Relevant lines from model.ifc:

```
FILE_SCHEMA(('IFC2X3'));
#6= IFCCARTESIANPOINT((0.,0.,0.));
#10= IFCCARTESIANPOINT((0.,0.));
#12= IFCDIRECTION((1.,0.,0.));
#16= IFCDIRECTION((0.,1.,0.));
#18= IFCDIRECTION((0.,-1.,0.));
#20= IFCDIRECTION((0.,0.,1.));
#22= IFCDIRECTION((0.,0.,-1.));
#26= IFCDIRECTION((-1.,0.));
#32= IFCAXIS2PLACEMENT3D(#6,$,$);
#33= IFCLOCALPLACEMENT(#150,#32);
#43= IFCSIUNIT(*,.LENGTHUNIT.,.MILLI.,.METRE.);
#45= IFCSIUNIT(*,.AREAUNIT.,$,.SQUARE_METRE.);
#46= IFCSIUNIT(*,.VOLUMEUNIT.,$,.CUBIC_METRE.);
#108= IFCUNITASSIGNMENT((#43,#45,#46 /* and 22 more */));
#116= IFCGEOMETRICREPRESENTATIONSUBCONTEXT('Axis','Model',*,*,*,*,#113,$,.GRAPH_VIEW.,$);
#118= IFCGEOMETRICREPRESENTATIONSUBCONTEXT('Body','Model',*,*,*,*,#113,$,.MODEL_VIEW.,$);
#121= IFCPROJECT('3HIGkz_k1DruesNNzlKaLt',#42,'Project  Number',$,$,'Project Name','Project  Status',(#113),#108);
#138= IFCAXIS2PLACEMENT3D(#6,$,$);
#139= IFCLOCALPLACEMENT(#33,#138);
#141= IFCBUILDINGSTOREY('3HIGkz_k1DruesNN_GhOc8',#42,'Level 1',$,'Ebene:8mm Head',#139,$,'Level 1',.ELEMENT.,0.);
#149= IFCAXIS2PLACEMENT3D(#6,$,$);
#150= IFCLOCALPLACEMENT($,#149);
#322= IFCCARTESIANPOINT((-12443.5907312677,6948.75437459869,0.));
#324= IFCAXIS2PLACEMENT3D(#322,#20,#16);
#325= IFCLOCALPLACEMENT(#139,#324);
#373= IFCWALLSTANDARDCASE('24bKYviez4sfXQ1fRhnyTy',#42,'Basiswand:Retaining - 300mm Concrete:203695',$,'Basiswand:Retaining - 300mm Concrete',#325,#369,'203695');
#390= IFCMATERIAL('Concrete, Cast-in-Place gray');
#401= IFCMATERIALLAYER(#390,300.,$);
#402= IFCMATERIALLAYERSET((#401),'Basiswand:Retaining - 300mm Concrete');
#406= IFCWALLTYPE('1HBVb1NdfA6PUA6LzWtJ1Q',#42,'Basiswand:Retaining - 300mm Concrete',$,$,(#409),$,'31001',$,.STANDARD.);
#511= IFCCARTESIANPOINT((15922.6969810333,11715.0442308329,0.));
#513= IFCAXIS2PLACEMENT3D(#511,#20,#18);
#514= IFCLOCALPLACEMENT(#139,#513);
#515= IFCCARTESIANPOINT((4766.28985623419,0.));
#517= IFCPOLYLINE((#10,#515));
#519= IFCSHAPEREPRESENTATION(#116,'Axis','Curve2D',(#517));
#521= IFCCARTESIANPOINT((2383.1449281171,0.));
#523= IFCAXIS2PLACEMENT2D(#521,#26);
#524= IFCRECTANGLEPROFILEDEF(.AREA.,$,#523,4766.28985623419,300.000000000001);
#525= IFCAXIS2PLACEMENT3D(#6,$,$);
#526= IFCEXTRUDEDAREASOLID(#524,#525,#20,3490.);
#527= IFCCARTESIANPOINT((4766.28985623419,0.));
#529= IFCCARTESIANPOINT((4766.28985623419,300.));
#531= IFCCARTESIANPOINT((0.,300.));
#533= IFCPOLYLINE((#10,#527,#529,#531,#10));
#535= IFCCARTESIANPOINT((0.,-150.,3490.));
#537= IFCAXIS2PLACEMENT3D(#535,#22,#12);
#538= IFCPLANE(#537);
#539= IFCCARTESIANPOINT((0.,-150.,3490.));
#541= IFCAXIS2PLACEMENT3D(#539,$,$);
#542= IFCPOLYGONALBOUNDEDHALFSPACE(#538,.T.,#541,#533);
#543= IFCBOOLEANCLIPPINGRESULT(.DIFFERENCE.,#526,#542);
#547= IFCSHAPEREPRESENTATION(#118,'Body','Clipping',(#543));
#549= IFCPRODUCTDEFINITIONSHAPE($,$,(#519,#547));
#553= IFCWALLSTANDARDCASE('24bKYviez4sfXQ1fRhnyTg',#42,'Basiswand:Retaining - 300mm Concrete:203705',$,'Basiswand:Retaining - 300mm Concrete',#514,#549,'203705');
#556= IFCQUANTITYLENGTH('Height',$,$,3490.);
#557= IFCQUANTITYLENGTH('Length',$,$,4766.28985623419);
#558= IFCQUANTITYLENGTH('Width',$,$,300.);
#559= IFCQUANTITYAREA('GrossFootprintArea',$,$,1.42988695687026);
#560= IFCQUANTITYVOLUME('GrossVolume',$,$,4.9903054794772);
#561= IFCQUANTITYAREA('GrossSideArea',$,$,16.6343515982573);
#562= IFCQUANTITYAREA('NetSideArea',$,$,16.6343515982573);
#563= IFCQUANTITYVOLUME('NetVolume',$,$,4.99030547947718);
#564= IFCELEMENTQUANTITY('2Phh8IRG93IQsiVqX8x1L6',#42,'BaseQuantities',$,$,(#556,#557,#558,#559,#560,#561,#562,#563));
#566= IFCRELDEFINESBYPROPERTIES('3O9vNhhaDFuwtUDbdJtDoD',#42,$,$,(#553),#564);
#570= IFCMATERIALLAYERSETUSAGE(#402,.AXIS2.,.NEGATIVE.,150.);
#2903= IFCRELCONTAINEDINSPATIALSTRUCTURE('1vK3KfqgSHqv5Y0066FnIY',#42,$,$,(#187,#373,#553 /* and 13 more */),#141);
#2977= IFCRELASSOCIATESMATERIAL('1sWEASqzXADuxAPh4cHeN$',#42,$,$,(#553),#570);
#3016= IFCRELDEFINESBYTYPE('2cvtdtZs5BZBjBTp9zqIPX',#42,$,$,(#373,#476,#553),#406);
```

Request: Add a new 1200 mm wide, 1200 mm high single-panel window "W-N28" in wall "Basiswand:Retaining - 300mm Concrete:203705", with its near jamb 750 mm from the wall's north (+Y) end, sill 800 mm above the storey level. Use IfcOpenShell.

```python
import numpy as np
import ifcopenshell
import ifcopenshell.api.feature
import ifcopenshell.api.geometry
import ifcopenshell.api.pset
import ifcopenshell.api.root
import ifcopenshell.api.spatial
import ifcopenshell.api.type
import ifcopenshell.geom
import ifcopenshell.util.element
import ifcopenshell.util.placement
import ifcopenshell.util.representation
import ifcopenshell.util.shape
import ifcopenshell.util.unit

model = ifcopenshell.open("model.ifc")
unit_scale = ifcopenshell.util.unit.calculate_unit_scale(model)
area_scale = ifcopenshell.util.unit.calculate_unit_scale(model, "AREAUNIT")
volume_scale = ifcopenshell.util.unit.calculate_unit_scale(model, "VOLUMEUNIT")
settings = ifcopenshell.geom.settings()


def volume(element):
    """Net volume in cubic metres, openings subtracted."""
    shape = ifcopenshell.geom.create_shape(settings, element)
    return ifcopenshell.util.shape.get_volume(shape.geometry)


wall = model.by_guid("24bKYviez4sfXQ1fRhnyTg")
storey = ifcopenshell.util.element.get_container(wall, ifc_class="IfcBuildingStorey")
context = ifcopenshell.util.representation.get_context(model, "Model", "Body", "MODEL_VIEW")
before = volume(wall)

width, height, from_end, sill = 1.2, 1.2, 0.75, 0.8  # metres

# The wall runs along its own X axis, and the end named is its -X end.
wall_shape = ifcopenshell.geom.create_shape(settings, wall)
x, y, z = ifcopenshell.util.shape.get_vertices(wall_shape.geometry).T
start = x.min() + from_end
face, thickness = float(y.min()), float(y.max() - y.min())
wall_matrix = ifcopenshell.util.placement.get_local_placement(wall.ObjectPlacement)
level = ifcopenshell.util.placement.get_local_placement(storey.ObjectPlacement)[2, 3]


def in_wall(x, y):
    """Placement at x, y metres in the wall's axes, at sill height."""
    matrix = wall_matrix.copy()
    matrix[:, 3] = wall_matrix @ np.array([x / unit_scale, y / unit_scale, 0.0, 1.0])
    matrix[2, 3] = level + sill / unit_scale
    return matrix


# Opening: a box that overshoots both wall faces by 50 mm.
opening = ifcopenshell.api.root.create_entity(model, ifc_class="IfcOpeningElement")
box = ifcopenshell.api.geometry.add_wall_representation(
    model, context=context, length=width, height=height, thickness=thickness + 0.1
)
ifcopenshell.api.geometry.assign_representation(model, product=opening, representation=box)
ifcopenshell.api.geometry.edit_object_placement(model, product=opening, matrix=in_wall(start, face - 0.05), is_si=False)
ifcopenshell.api.feature.add_feature(model, feature=opening, element=wall)

window = ifcopenshell.api.root.create_entity(model, ifc_class="IfcWindow", name="W-N28")
window.OverallWidth, window.OverallHeight = width / unit_scale, height / unit_scale
body = ifcopenshell.api.geometry.add_window_representation(
    model,
    context=context,
    overall_width=window.OverallWidth,
    overall_height=window.OverallHeight,
    partition_type="SINGLE_PANEL",
)
ifcopenshell.api.geometry.assign_representation(model, product=window, representation=body)
ifcopenshell.api.spatial.assign_container(model, products=[window], relating_structure=storey)
fills = ifcopenshell.api.feature.add_filling(model, opening=opening, element=window)
fills.OwnerHistory = window.OwnerHistory  # required in IFC2X3

# IFC2X3 keeps the operation on the window style.
style = ifcopenshell.api.root.create_entity(model, ifc_class="IfcWindowStyle", name="W-N28")
style.OperationType, style.ConstructionType = "SINGLE_PANEL", "NOTDEFINED"
style.ParameterTakesPrecedence = style.Sizeable = False
ifcopenshell.api.type.assign_type(model, related_objects=[window], relating_type=style)

# Centre the window in the wall's thickness.
ifcopenshell.api.geometry.edit_object_placement(model, product=window, matrix=in_wall(start, face), is_si=False)
window_shape = ifcopenshell.geom.create_shape(settings, window)
depth = ifcopenshell.util.shape.get_vertices(window_shape.geometry)[:, 1]
offset = face + thickness / 2 - (depth.min() + depth.max()) / 2
ifcopenshell.api.geometry.edit_object_placement(model, product=window, matrix=in_wall(start, offset), is_si=False)

after = volume(wall)

# Update the wall's stored quantities.
qto = model.by_id(ifcopenshell.util.element.get_pset(wall, "BaseQuantities", should_inherit=False)["id"])
ifcopenshell.api.pset.edit_qto(model, qto=qto, properties={
    "NetSideArea": after / thickness / area_scale,
    "NetVolume": after / volume_scale,
})

print(f"wall volume {before:.3f} -> {after:.3f} m3")

model.write("model_rev.ifc")
```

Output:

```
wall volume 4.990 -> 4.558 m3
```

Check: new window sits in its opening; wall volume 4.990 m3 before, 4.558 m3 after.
